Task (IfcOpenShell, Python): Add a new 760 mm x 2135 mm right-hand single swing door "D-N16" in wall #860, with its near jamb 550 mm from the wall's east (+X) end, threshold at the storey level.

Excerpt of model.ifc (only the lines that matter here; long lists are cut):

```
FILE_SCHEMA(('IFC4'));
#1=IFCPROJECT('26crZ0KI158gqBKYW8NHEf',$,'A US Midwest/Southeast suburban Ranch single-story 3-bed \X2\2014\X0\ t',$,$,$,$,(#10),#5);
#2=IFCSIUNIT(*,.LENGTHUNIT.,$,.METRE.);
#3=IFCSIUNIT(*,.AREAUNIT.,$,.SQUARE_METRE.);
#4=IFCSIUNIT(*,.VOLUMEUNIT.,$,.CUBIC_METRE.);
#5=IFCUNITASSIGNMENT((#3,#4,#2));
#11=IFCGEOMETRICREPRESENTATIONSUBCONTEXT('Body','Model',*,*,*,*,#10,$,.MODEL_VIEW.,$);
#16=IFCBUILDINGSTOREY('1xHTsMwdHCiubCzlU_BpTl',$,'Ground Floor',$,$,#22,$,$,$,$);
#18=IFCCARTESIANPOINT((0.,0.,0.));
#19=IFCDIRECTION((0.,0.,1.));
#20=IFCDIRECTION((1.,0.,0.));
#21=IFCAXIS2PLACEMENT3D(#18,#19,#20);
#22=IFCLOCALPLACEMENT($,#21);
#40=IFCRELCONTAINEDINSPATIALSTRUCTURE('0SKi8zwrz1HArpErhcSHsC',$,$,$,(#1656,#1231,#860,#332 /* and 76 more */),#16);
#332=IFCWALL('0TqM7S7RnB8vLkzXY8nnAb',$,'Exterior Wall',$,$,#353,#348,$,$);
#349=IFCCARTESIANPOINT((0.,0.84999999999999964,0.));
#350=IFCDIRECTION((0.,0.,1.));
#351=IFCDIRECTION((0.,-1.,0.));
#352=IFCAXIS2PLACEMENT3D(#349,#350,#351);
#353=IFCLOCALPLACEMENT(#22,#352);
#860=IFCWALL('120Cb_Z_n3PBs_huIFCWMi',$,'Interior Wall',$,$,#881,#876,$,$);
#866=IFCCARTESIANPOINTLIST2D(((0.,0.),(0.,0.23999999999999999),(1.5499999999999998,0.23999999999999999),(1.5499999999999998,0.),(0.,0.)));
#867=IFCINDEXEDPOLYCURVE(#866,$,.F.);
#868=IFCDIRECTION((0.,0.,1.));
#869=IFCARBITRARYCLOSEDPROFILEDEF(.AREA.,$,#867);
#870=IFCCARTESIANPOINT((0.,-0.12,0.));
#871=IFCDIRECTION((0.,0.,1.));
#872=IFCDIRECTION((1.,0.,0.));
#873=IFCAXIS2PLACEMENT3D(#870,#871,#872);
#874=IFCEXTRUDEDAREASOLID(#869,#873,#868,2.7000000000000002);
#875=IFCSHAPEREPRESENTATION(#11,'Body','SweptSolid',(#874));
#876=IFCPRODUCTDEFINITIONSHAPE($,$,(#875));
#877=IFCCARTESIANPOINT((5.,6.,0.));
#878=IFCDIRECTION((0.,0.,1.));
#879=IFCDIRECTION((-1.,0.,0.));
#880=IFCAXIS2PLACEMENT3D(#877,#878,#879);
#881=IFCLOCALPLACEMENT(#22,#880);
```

```python
import numpy as np
import ifcopenshell
import ifcopenshell.api.feature
import ifcopenshell.api.geometry
import ifcopenshell.api.root
import ifcopenshell.api.spatial
import ifcopenshell.geom
import ifcopenshell.util.element
import ifcopenshell.util.placement
import ifcopenshell.util.representation
import ifcopenshell.util.shape
import ifcopenshell.util.unit

model = ifcopenshell.open("model.ifc")
unit_scale = ifcopenshell.util.unit.calculate_unit_scale(model)
settings = ifcopenshell.geom.settings()


def volume(element):
    """Net volume in cubic metres, openings subtracted."""
    shape = ifcopenshell.geom.create_shape(settings, element)
    return ifcopenshell.util.shape.get_volume(shape.geometry)


wall = model.by_guid("120Cb_Z_n3PBs_huIFCWMi")
storey = ifcopenshell.util.element.get_container(wall, ifc_class="IfcBuildingStorey")
context = ifcopenshell.util.representation.get_context(model, "Model", "Body", "MODEL_VIEW")
before = volume(wall)

width, height, from_end, sill = 0.76, 2.135, 0.55, 0.0  # metres

# The wall runs along its own X axis, and the end named is its -X end.
wall_shape = ifcopenshell.geom.create_shape(settings, wall)
x, y, z = ifcopenshell.util.shape.get_vertices(wall_shape.geometry).T
start = x.min() + from_end
face, thickness = float(y.min()), float(y.max() - y.min())
wall_matrix = ifcopenshell.util.placement.get_local_placement(wall.ObjectPlacement)
level = ifcopenshell.util.placement.get_local_placement(storey.ObjectPlacement)[2, 3]


def in_wall(x, y):
    """Placement at x, y metres in the wall's axes, at sill height."""
    matrix = wall_matrix.copy()
    matrix[:, 3] = wall_matrix @ np.array([x / unit_scale, y / unit_scale, 0.0, 1.0])
    matrix[2, 3] = level + sill / unit_scale
    return matrix


# Opening: a box that overshoots both wall faces by 50 mm.
opening = ifcopenshell.api.root.create_entity(model, ifc_class="IfcOpeningElement", predefined_type="OPENING")
box = ifcopenshell.api.geometry.add_wall_representation(
    model, context=context, length=width, height=height, thickness=thickness + 0.1
)
ifcopenshell.api.geometry.assign_representation(model, product=opening, representation=box)
ifcopenshell.api.geometry.edit_object_placement(model, product=opening, matrix=in_wall(start, face - 0.05), is_si=False)
ifcopenshell.api.feature.add_feature(model, feature=opening, element=wall)

door = ifcopenshell.api.root.create_entity(model, ifc_class="IfcDoor", name="D-N16", predefined_type="DOOR")
door.OverallWidth, door.OverallHeight = width / unit_scale, height / unit_scale
door.OperationType = "SINGLE_SWING_RIGHT"
body = ifcopenshell.api.geometry.add_door_representation(
    model,
    context=context,
    overall_width=door.OverallWidth,
    overall_height=door.OverallHeight,
    operation_type="SINGLE_SWING_RIGHT",
    lining_properties={"LiningDepth": thickness / unit_scale, "ThresholdDepth": thickness / unit_scale},
)
ifcopenshell.api.geometry.assign_representation(model, product=door, representation=body)
ifcopenshell.api.spatial.assign_container(model, products=[door], relating_structure=storey)
ifcopenshell.api.feature.add_filling(model, opening=opening, element=door)

# The lining spans the wall, so the door starts at the wall face.
ifcopenshell.api.geometry.edit_object_placement(model, product=door, matrix=in_wall(start, face), is_si=False)

after = volume(wall)

print(f"wall volume {before:.3f} -> {after:.3f} m3")

model.write("model-out.ifc")
```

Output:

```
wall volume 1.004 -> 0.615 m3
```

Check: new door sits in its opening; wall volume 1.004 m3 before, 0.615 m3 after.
